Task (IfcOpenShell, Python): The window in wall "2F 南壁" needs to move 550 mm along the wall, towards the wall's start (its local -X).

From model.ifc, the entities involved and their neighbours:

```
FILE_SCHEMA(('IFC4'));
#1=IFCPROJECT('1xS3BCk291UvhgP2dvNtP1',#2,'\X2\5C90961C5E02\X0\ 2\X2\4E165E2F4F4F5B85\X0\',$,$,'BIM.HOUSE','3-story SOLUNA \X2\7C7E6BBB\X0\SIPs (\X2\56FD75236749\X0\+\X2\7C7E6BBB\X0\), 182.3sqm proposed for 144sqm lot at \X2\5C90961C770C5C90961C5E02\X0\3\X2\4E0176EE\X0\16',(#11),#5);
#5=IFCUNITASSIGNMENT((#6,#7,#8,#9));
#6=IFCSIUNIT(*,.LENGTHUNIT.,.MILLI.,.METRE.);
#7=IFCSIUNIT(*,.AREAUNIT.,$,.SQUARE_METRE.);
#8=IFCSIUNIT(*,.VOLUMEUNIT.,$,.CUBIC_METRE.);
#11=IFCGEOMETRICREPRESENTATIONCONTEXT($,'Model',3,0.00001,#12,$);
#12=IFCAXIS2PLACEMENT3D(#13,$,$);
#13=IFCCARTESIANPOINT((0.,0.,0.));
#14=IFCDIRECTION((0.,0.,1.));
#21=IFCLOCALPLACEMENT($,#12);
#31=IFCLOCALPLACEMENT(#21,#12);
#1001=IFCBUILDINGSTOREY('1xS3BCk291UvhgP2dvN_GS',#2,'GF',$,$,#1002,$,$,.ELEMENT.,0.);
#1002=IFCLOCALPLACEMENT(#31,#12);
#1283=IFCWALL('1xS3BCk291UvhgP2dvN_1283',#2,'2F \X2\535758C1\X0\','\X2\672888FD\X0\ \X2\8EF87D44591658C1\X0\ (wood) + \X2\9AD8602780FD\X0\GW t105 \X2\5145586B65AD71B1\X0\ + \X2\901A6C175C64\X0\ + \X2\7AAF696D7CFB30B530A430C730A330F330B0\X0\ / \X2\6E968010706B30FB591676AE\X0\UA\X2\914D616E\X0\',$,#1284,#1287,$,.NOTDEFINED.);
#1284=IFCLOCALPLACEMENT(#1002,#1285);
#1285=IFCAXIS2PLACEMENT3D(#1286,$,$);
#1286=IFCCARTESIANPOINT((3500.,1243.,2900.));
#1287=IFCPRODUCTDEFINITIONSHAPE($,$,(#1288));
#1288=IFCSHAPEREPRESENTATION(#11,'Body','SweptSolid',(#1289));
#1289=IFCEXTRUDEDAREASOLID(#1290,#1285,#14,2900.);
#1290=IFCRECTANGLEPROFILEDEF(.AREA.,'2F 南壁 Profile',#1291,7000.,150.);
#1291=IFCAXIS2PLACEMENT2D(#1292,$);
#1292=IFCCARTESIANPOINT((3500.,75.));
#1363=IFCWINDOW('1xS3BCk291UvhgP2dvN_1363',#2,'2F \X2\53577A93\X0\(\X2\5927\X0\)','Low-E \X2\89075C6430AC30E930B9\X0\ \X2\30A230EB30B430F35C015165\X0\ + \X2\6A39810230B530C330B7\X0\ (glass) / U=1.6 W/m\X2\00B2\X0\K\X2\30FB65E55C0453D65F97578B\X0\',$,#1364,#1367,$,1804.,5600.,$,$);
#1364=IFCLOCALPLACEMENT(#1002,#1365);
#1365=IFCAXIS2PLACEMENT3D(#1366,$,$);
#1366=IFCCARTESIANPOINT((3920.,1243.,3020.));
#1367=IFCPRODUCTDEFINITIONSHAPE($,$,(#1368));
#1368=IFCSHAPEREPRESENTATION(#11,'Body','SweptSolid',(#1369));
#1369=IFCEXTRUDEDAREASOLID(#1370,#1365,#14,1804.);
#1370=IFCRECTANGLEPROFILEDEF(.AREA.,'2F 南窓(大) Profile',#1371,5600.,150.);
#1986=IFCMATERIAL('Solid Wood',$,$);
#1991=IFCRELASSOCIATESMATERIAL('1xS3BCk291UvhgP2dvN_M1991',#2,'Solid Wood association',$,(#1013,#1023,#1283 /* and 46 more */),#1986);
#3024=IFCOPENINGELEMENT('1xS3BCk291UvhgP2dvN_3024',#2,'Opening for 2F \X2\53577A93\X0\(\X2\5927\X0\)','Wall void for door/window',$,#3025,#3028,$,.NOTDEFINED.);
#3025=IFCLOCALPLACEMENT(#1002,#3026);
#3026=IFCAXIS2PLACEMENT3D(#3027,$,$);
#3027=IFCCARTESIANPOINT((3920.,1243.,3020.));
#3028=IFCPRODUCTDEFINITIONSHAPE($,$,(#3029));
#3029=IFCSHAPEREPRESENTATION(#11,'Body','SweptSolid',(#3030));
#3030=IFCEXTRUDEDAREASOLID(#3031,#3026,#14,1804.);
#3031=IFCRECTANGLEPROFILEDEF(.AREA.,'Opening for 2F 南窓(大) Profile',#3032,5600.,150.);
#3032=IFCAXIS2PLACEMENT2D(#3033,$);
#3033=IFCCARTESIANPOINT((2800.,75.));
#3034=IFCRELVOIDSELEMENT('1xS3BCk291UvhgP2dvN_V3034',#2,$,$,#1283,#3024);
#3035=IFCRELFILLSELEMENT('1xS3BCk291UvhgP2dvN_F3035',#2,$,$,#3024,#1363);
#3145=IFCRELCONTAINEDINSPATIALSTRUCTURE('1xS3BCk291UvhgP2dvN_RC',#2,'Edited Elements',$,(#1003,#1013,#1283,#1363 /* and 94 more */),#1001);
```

```python
import ifcopenshell
import ifcopenshell.api.geometry
import ifcopenshell.util.placement

model = ifcopenshell.open("model.ifc")

window = model.by_guid("1xS3BCk291UvhgP2dvN_1363")
opening = window.FillsVoids[0].RelatingOpeningElement
wall = opening.VoidsElements[0].RelatingBuildingElement

wall_matrix = ifcopenshell.util.placement.get_local_placement(wall.ObjectPlacement)
shift = wall_matrix[:3, 0] * -550.0
before = ifcopenshell.util.placement.get_local_placement(window.ObjectPlacement)[:3, 3].copy()

# The window is not placed relative to its opening, so move both.
for product in (opening, window):
    matrix = ifcopenshell.util.placement.get_local_placement(product.ObjectPlacement)
    matrix[:3, 3] += shift
    ifcopenshell.api.geometry.edit_object_placement(model, product=product, matrix=matrix, is_si=False)

after = ifcopenshell.util.placement.get_local_placement(window.ObjectPlacement)[:3, 3]
print("window moved by", (after - before).round(3) + 0.0)

model.write("model_v2.ifc")
```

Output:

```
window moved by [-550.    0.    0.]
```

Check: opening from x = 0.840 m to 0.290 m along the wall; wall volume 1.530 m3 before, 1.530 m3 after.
